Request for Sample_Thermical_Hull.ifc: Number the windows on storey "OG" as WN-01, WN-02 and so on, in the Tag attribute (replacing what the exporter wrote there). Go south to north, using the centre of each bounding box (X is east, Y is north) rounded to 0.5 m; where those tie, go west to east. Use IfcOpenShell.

First a look at what the model holds.

```python
import ifcopenshell
import ifcopenshell.util.element
import ifcopenshell.util.placement

model = ifcopenshell.open("Sample_Thermical_Hull.ifc")
print(model.schema)
storey = next(s for s in model.by_type("IfcBuildingStorey") if s.Name == "OG")
windows = [e for e in ifcopenshell.util.element.get_decomposition(storey) if e.is_a("IfcWindow")]
for e in sorted(windows, key=lambda e: e.id()):
    origin = ifcopenshell.util.placement.get_local_placement(e.ObjectPlacement)[:3, 3]
    print(e.id(), e.Tag, e.Name, origin.round(2) + 0.0, sep=" | ")
```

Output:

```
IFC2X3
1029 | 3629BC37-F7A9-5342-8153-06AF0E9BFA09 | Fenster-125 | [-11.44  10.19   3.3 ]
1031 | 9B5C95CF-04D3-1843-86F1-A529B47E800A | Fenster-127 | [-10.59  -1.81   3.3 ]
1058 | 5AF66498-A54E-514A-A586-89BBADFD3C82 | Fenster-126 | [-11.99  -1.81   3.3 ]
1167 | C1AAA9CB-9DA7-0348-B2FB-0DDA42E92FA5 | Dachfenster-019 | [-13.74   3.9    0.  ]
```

```python
import ifcopenshell
import ifcopenshell.geom
import ifcopenshell.util.element
import ifcopenshell.util.shape

model = ifcopenshell.open("Sample_Thermical_Hull.ifc")
settings = ifcopenshell.geom.settings()
settings.set("use-world-coords", True)


def centre(element):
    shape = ifcopenshell.geom.create_shape(settings, element)
    return ifcopenshell.util.shape.get_bbox_centroid(shape.geometry)


storey = next(s for s in model.by_type("IfcBuildingStorey") if s.Name == "OG")
windows = [e for e in ifcopenshell.util.element.get_decomposition(storey) if e.is_a("IfcWindow")]

# Insertion points can sit at a corner or the storey origin, so sort by the geometry (in metres).
centres = {e: centre(e) for e in windows}
windows.sort(key=lambda e: (round(centres[e][1] / 0.5), centres[e][0]))

for i, e in enumerate(windows, start=1):
    number = f"WN-{i:02d}"
    e.Tag = number
    print(e.id(), number)

model.write("Sample_Thermical_Hull-out.ifc")
```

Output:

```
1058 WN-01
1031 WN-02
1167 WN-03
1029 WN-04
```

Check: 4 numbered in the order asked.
